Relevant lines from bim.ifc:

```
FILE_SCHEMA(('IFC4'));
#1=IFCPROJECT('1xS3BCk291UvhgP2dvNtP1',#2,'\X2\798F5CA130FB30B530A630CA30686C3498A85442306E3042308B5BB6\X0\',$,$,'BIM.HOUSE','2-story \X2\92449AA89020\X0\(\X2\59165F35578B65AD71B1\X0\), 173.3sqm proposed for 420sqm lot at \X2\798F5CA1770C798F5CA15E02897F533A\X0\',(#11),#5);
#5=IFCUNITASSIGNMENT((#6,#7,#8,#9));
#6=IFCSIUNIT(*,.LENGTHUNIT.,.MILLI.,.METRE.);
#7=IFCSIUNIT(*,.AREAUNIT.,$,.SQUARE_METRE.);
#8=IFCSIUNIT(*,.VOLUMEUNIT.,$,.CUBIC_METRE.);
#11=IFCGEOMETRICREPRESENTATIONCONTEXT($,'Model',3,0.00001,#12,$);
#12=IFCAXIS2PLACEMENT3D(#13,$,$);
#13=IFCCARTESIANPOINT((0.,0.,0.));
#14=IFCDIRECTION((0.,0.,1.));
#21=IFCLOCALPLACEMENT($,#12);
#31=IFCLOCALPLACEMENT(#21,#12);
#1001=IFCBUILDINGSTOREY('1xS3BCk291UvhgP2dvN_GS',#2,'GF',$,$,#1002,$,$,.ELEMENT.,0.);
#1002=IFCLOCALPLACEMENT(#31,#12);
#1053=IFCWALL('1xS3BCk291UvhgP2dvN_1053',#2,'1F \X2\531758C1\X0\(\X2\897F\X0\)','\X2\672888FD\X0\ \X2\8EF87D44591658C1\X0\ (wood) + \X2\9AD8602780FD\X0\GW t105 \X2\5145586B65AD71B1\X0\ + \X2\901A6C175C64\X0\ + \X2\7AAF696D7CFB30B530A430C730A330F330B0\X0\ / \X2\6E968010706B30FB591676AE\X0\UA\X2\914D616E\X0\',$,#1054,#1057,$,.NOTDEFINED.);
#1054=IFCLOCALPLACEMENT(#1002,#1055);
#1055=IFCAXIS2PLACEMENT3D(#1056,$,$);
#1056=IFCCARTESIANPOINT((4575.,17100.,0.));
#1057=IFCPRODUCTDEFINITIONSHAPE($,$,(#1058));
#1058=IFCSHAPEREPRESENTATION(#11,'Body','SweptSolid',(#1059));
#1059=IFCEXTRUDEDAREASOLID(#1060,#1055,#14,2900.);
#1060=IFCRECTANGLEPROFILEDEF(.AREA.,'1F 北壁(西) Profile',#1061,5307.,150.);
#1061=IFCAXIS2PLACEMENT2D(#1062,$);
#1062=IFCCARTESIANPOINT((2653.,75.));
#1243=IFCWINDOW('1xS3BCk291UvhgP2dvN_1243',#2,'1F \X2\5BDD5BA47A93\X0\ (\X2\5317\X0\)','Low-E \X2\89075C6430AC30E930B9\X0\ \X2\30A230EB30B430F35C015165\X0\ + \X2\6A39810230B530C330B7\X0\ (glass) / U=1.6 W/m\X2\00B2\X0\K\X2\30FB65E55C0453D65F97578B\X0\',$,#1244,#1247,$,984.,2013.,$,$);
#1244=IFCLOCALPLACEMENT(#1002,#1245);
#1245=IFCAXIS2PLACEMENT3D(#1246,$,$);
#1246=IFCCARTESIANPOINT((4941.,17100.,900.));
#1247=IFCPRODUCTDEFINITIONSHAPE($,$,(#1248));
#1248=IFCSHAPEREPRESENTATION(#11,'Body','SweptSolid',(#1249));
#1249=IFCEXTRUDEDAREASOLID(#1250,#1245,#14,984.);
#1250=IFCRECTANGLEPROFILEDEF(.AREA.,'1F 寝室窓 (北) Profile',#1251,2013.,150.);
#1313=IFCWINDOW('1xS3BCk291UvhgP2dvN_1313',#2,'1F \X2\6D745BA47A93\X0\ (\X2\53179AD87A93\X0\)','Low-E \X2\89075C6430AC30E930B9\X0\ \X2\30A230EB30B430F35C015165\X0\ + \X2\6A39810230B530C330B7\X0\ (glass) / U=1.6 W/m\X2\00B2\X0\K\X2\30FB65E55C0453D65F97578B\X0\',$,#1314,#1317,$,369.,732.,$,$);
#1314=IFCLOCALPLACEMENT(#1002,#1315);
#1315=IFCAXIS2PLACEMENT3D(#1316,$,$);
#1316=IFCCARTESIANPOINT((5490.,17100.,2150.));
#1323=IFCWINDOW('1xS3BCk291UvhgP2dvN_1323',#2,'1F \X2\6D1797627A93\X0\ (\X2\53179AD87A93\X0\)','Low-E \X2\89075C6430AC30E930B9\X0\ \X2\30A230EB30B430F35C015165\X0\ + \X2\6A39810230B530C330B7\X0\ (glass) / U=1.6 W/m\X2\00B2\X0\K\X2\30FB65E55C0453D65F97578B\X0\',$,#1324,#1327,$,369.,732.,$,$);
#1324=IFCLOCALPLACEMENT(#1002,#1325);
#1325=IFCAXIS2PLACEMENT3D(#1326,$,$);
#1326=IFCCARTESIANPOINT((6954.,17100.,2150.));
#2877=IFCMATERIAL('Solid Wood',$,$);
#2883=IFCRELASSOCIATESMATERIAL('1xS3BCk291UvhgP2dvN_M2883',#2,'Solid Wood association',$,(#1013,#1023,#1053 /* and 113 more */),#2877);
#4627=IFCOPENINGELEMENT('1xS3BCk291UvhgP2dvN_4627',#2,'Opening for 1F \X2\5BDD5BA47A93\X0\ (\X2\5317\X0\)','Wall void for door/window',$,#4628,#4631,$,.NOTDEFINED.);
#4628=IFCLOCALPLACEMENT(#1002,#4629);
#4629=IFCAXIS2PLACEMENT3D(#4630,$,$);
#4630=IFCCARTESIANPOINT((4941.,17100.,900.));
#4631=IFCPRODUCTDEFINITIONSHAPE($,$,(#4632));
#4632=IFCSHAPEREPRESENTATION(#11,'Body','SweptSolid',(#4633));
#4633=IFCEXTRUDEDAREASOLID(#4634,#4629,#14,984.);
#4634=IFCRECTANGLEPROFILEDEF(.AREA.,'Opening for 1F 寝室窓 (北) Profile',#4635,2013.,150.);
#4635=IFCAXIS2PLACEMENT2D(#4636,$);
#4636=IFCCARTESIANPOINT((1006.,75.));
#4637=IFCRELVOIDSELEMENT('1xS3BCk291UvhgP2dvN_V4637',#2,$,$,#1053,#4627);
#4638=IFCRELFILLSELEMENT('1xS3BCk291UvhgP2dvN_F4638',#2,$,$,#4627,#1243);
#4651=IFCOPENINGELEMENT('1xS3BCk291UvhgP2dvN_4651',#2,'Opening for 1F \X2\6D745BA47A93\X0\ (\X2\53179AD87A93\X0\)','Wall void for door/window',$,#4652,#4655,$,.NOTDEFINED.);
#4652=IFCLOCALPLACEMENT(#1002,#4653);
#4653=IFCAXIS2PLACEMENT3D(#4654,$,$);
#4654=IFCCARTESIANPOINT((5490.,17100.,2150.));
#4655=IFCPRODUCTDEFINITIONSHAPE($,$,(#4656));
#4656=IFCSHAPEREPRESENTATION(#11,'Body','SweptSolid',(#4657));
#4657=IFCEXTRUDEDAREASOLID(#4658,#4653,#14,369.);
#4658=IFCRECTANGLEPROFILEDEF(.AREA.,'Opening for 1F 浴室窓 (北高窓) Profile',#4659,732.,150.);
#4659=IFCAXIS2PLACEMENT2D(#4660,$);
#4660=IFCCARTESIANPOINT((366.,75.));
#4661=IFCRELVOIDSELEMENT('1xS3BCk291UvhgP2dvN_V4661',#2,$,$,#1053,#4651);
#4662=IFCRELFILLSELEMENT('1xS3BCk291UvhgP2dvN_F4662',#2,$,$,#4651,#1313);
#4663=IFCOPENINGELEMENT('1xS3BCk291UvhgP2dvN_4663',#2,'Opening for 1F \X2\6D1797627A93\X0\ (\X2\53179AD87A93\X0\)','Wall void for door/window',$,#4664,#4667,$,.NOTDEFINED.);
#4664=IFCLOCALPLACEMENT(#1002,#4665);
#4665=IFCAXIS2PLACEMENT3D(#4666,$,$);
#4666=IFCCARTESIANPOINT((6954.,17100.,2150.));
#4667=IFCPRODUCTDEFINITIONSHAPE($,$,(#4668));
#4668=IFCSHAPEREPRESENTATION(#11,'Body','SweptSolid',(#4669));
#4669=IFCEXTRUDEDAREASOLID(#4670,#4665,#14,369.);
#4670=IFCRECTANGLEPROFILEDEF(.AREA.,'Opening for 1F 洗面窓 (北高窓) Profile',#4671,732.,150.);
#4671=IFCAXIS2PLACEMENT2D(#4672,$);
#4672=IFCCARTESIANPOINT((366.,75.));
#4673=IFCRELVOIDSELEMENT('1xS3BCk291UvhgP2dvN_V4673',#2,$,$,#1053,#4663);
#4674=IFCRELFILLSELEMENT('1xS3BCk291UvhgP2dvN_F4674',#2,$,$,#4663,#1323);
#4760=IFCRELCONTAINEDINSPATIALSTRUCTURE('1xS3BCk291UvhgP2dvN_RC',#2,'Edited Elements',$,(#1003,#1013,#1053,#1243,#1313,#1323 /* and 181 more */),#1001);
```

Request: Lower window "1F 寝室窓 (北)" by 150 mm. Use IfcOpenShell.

```python
import numpy as np
import ifcopenshell
import ifcopenshell.api.geometry
import ifcopenshell.util.placement
import ifcopenshell.util.unit

model = ifcopenshell.open("bim.ifc")
unit_scale = ifcopenshell.util.unit.calculate_unit_scale(model)

window = model.by_guid("1xS3BCk291UvhgP2dvN_1243")
opening = window.FillsVoids[0].RelatingOpeningElement
dz = -0.15 / unit_scale

shift = np.array([0.0, 0.0, dz])
# The window is not placed relative to its opening, so move both.
for product in (opening, window):
    matrix = ifcopenshell.util.placement.get_local_placement(product.ObjectPlacement)
    matrix[:3, 3] += shift
    ifcopenshell.api.geometry.edit_object_placement(model, product=product, matrix=matrix, is_si=False)

print(f"moved by {dz * unit_scale:+.3f} m")

model.write("bim_rev.ifc")
```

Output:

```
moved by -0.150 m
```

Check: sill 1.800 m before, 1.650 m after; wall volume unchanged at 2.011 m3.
